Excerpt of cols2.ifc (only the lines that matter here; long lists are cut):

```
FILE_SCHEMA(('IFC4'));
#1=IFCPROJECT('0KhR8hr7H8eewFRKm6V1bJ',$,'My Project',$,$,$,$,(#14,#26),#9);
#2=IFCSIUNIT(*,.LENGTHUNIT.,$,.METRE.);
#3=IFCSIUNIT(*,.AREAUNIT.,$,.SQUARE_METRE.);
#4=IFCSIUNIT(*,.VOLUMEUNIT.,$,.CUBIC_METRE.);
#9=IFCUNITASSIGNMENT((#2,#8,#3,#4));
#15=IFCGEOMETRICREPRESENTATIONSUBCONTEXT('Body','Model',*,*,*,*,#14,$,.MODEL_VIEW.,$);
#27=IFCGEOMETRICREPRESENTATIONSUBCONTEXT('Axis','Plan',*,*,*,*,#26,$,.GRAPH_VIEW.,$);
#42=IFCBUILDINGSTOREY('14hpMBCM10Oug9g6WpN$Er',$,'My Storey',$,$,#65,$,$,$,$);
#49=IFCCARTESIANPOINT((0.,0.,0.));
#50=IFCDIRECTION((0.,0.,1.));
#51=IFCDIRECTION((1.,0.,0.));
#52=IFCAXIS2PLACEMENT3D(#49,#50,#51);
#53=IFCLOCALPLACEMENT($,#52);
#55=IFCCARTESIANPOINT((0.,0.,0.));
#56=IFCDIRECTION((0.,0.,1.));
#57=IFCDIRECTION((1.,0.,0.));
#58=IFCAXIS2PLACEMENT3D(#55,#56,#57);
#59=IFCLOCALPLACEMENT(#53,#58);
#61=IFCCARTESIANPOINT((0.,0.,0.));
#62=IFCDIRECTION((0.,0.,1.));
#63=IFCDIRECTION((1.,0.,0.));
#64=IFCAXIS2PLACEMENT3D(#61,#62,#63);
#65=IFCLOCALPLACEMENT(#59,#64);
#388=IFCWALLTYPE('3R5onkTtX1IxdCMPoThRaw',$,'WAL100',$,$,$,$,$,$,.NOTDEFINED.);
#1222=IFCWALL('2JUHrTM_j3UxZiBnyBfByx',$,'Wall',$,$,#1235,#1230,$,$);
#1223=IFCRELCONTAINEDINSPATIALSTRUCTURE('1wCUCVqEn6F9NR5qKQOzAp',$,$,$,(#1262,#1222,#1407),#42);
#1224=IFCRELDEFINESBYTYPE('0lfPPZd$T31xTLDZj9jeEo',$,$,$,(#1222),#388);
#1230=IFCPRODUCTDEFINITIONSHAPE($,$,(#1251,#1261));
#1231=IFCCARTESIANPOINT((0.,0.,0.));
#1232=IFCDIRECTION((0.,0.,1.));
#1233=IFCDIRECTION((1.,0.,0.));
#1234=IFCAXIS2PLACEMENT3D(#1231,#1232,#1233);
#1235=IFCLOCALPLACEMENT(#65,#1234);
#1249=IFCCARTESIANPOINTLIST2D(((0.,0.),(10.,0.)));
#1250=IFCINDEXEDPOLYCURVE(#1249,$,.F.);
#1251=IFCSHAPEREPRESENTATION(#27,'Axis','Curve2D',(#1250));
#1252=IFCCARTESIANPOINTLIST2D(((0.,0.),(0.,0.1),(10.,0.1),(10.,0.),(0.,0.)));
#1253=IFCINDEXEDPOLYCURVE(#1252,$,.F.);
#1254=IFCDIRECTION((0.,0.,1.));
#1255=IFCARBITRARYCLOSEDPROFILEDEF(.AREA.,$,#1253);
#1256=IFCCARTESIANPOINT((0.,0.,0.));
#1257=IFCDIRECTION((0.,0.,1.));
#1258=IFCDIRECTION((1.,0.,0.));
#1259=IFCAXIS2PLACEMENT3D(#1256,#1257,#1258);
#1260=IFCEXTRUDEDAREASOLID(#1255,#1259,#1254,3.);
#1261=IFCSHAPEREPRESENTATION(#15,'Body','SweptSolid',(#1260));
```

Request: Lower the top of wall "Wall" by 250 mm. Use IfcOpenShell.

```python
import ifcopenshell
import ifcopenshell.geom
import ifcopenshell.util.representation
import ifcopenshell.util.shape

model = ifcopenshell.open("cols2.ifc")
settings = ifcopenshell.geom.settings()


def volume(element):
    """Net volume in cubic metres, openings subtracted."""
    shape = ifcopenshell.geom.create_shape(settings, element)
    return ifcopenshell.util.shape.get_volume(shape.geometry)


wall = model.by_guid("2JUHrTM_j3UxZiBnyBfByx")
before = volume(wall)

body = ifcopenshell.util.representation.get_representation(wall, "Model", "Body")
solid = body.Items[0]
old_height = solid.Depth
solid.Depth -= 0.25
after = volume(wall)

print(f"height {old_height:g} -> {solid.Depth:g}, volume {before:.3f} -> {after:.3f} m3")

model.write("cols2_updated.ifc")
```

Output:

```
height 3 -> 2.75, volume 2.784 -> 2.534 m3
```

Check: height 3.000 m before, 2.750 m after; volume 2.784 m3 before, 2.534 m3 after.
